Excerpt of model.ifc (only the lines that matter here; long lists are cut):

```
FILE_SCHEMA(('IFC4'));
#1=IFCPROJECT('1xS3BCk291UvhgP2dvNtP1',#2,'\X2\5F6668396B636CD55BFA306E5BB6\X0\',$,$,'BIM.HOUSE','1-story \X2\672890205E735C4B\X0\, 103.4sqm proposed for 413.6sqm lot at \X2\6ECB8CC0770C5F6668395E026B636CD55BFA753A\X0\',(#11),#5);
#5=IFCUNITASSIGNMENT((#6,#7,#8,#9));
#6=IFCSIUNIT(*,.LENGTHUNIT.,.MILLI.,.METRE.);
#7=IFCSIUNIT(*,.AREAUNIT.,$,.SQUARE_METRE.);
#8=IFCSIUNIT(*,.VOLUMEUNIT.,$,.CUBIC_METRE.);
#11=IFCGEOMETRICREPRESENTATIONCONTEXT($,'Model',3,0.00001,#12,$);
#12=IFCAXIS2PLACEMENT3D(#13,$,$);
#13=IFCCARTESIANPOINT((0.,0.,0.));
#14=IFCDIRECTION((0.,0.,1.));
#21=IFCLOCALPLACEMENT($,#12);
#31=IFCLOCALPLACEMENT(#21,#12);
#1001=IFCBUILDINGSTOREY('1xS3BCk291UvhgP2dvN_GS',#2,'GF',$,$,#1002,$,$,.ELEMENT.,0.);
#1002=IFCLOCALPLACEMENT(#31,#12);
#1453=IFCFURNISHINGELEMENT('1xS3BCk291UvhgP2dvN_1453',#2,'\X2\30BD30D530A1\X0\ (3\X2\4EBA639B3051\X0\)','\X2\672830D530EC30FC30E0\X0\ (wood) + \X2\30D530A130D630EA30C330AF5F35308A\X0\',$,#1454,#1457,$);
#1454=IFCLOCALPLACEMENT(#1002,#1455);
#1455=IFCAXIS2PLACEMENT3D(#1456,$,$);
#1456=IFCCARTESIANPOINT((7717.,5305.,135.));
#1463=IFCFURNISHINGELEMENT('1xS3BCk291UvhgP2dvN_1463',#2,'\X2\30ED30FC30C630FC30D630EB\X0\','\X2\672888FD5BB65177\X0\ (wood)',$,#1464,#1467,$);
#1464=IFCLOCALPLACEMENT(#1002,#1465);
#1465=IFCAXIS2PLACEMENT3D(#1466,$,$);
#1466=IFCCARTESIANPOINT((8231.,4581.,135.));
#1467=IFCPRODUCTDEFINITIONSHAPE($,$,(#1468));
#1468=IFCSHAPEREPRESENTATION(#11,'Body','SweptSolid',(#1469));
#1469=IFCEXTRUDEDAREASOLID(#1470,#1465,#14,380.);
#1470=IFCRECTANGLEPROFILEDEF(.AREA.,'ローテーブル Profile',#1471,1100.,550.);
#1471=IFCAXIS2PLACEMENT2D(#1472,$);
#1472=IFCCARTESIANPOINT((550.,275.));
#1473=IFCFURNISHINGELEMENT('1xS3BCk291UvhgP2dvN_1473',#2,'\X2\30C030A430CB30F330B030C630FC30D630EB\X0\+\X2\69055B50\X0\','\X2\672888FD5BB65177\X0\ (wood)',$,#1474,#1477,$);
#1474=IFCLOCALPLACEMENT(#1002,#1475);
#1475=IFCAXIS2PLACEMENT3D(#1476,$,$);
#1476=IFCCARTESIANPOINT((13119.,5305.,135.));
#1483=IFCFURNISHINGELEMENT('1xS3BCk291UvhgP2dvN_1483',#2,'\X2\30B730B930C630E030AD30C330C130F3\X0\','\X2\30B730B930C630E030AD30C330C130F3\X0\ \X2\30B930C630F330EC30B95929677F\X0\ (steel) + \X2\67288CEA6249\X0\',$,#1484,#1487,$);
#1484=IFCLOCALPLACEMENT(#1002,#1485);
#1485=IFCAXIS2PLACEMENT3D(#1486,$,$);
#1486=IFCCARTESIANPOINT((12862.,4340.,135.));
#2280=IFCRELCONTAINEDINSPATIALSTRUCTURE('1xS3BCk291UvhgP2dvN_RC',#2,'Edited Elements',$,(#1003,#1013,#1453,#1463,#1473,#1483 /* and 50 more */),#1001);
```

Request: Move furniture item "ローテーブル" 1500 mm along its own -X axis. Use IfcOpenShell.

```python
import ifcopenshell
import ifcopenshell.api.geometry
import ifcopenshell.util.placement
import ifcopenshell.util.unit

model = ifcopenshell.open("model.ifc")
unit_scale = ifcopenshell.util.unit.calculate_unit_scale(model)

item = model.by_guid("1xS3BCk291UvhgP2dvN_1463")
matrix = ifcopenshell.util.placement.get_local_placement(item.ObjectPlacement)
matrix[:3, 3] -= matrix[:3, 0] * 1.5 / unit_scale
ifcopenshell.api.geometry.edit_object_placement(model, product=item, matrix=matrix, is_si=False)

print(ifcopenshell.util.placement.get_local_placement(item.ObjectPlacement).round(3) + 0.0)

model.write("model_v2.ifc")
```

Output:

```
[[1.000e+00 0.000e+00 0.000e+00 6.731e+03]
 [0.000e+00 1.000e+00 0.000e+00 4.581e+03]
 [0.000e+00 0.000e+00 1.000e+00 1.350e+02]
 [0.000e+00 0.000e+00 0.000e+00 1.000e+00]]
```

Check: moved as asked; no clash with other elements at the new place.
